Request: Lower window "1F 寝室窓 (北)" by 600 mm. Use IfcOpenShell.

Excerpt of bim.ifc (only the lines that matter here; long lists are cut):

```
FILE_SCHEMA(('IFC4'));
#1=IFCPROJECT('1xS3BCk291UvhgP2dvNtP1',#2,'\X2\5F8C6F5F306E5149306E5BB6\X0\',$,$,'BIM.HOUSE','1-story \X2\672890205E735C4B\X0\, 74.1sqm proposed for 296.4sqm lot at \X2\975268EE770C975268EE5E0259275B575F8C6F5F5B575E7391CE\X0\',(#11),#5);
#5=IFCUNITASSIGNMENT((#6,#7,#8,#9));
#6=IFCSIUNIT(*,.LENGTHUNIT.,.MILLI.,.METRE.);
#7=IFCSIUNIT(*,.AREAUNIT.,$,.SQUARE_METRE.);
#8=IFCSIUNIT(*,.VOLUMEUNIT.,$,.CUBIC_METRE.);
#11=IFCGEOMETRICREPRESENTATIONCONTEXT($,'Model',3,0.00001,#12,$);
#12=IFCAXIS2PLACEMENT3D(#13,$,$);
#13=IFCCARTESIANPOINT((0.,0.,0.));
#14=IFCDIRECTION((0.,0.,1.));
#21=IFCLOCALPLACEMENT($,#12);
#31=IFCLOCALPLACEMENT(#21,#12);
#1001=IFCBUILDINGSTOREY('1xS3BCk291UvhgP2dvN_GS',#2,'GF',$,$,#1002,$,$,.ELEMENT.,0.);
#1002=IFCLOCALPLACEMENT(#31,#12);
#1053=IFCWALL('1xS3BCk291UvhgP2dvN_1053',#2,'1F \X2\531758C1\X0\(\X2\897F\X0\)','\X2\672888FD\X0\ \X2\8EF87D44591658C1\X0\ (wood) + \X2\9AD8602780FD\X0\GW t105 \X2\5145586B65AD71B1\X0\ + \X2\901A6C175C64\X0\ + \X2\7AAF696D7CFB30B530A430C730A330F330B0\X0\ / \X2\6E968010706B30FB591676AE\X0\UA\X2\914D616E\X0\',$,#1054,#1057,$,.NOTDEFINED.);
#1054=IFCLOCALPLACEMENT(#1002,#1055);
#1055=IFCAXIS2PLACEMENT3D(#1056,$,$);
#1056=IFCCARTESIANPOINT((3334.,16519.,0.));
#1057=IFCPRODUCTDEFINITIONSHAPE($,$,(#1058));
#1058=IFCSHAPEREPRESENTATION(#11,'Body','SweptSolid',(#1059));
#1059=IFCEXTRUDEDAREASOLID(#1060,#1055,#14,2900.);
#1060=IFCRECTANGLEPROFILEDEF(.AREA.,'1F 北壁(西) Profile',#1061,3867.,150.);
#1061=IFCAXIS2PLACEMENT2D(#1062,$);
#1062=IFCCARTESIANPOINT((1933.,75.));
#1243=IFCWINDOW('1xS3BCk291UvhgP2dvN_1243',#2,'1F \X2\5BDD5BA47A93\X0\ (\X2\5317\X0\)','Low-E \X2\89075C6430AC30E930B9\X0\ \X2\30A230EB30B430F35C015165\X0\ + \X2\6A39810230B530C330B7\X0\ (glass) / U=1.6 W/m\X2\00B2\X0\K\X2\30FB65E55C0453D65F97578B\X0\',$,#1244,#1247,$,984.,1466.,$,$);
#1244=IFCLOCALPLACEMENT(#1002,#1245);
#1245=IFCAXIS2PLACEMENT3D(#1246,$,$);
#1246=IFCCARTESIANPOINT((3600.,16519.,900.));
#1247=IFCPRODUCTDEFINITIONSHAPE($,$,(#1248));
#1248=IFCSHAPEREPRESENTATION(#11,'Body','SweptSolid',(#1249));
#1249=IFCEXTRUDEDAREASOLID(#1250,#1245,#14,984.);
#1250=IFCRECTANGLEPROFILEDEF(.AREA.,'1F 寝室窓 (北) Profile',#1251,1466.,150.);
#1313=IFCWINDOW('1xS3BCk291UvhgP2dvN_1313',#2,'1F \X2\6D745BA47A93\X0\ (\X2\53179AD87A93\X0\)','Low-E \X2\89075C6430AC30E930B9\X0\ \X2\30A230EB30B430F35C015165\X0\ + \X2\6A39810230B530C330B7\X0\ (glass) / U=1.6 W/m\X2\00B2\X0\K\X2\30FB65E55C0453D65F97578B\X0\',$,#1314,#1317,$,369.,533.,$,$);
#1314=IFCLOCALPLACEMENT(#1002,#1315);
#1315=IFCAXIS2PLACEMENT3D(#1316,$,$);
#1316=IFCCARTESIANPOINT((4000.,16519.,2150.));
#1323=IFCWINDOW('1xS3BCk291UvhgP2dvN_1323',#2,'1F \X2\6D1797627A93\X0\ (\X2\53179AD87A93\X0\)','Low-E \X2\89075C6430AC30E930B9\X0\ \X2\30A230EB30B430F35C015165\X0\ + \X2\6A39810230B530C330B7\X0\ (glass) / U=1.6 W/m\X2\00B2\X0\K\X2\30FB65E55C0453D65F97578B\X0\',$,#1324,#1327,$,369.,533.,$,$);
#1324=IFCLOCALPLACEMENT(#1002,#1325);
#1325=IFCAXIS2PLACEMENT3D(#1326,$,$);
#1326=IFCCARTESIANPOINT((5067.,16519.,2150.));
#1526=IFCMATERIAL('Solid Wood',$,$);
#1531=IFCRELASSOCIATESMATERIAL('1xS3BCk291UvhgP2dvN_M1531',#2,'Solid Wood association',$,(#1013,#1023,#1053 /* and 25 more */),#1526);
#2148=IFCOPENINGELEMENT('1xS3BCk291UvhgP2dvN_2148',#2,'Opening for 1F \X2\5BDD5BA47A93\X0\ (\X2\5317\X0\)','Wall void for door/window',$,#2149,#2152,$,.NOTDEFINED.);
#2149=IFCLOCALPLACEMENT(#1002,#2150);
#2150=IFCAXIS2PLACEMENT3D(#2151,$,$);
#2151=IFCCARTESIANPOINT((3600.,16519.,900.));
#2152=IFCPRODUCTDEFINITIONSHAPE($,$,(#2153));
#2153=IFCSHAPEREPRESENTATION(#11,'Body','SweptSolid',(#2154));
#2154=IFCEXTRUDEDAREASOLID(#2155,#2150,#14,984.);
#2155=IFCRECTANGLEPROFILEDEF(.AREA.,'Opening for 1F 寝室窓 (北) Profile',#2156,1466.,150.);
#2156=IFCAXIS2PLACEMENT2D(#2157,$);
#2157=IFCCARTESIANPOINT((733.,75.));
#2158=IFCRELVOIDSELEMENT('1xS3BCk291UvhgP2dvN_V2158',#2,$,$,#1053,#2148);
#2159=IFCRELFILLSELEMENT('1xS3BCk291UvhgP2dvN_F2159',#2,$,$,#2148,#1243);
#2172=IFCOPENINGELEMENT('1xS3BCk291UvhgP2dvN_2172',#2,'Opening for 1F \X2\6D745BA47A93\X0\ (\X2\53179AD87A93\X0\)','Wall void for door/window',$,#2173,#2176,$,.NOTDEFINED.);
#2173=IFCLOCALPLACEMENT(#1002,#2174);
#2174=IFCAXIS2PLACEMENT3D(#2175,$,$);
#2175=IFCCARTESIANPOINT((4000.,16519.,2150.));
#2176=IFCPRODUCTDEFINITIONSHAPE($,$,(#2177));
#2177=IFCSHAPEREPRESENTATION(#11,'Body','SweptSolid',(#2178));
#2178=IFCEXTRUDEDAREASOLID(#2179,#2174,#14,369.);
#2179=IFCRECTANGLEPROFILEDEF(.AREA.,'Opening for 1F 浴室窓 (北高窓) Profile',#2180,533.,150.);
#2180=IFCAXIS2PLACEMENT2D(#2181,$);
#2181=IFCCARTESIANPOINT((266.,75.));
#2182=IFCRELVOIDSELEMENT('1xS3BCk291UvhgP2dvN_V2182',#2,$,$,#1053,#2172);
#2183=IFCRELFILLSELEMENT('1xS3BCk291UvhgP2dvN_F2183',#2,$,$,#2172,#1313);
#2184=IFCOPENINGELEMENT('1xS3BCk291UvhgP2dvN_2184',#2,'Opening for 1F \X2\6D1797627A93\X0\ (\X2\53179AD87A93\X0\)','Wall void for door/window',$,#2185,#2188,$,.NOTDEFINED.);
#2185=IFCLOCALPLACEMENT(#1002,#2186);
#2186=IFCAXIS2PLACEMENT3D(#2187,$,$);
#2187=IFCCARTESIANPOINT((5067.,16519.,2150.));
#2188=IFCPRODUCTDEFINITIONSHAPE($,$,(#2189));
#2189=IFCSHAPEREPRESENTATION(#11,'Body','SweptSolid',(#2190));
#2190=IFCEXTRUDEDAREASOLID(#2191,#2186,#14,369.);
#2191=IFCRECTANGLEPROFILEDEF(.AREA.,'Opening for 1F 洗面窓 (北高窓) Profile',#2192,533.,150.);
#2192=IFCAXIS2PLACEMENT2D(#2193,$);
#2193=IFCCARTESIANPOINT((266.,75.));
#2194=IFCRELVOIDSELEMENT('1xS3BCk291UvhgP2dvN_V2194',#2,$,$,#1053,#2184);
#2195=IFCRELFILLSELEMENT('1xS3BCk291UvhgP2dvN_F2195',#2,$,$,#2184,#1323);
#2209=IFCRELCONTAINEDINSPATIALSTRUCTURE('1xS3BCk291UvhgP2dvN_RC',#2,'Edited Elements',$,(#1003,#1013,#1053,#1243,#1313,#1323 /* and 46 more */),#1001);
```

```python
import numpy as np
import ifcopenshell
import ifcopenshell.api.geometry
import ifcopenshell.util.placement
import ifcopenshell.util.unit

model = ifcopenshell.open("bim.ifc")
unit_scale = ifcopenshell.util.unit.calculate_unit_scale(model)

window = model.by_guid("1xS3BCk291UvhgP2dvN_1243")
opening = window.FillsVoids[0].RelatingOpeningElement
dz = -600.0

shift = np.array([0.0, 0.0, dz])
# The window is not placed relative to its opening, so move both.
for product in (opening, window):
    matrix = ifcopenshell.util.placement.get_local_placement(product.ObjectPlacement)
    matrix[:3, 3] += shift
    ifcopenshell.api.geometry.edit_object_placement(model, product=product, matrix=matrix, is_si=False)

print(f"moved by {dz * unit_scale:+.3f} m")

model.write("bim_updated.ifc")
```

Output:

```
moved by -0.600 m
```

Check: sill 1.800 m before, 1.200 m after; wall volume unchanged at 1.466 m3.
